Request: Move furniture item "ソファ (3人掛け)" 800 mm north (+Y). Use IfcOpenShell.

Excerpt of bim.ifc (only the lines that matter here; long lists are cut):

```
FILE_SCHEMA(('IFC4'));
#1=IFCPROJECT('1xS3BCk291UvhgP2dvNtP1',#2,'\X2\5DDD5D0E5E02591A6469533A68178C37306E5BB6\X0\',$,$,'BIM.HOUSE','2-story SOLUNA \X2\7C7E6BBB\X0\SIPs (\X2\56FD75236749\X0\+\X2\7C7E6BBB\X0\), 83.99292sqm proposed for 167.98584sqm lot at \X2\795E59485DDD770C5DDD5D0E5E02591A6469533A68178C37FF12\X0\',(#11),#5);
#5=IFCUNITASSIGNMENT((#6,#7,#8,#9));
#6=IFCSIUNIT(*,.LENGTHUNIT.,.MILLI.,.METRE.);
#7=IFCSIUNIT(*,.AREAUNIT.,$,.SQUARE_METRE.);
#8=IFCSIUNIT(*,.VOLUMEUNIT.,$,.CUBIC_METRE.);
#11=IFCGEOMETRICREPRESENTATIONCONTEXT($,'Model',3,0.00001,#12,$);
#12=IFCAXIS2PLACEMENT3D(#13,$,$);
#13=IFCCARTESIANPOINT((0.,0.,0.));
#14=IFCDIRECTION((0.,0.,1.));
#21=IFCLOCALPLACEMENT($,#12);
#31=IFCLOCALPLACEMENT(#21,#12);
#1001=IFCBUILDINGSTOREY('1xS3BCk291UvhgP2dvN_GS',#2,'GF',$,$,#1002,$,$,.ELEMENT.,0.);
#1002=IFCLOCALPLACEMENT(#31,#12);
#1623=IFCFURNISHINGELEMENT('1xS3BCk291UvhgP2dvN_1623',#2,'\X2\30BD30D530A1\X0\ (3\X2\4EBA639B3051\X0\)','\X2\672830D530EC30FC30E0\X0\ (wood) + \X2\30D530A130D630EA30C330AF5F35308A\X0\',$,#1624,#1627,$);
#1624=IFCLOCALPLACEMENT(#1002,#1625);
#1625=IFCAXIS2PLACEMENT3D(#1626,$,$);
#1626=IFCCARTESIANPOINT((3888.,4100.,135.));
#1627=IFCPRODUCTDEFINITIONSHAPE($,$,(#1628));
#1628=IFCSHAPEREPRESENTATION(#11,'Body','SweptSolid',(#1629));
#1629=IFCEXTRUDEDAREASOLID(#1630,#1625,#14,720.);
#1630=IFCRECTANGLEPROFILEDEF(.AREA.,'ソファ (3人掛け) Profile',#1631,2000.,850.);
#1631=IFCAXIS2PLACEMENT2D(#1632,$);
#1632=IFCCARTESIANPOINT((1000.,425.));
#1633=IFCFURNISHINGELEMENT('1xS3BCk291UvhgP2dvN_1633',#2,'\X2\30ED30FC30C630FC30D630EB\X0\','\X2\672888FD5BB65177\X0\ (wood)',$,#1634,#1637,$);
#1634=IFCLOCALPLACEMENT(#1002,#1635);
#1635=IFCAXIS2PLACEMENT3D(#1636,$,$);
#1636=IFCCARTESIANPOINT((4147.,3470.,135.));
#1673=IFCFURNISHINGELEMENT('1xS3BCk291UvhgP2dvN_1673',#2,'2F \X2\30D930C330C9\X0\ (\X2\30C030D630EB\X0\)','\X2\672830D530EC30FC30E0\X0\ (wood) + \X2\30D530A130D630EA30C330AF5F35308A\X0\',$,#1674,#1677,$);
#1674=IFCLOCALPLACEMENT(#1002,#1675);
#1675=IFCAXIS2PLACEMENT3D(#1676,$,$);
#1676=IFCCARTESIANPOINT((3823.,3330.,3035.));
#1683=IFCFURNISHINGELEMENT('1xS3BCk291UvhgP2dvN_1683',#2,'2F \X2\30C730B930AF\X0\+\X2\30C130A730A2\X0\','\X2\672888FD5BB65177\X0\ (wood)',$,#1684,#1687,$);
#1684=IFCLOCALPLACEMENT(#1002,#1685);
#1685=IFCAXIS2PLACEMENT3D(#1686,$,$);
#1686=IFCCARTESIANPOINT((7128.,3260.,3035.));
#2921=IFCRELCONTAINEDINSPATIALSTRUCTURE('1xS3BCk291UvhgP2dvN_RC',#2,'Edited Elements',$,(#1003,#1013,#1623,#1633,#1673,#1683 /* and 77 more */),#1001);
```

```python
import ifcopenshell
import ifcopenshell.api.geometry
import ifcopenshell.util.placement
import ifcopenshell.util.unit

model = ifcopenshell.open("bim.ifc")
unit_scale = ifcopenshell.util.unit.calculate_unit_scale(model)

item = model.by_guid("1xS3BCk291UvhgP2dvN_1623")
matrix = ifcopenshell.util.placement.get_local_placement(item.ObjectPlacement)
matrix[1, 3] += 0.8 / unit_scale
ifcopenshell.api.geometry.edit_object_placement(model, product=item, matrix=matrix, is_si=False)

print(ifcopenshell.util.placement.get_local_placement(item.ObjectPlacement).round(3) + 0.0)

model.write("bim_edited.ifc")
```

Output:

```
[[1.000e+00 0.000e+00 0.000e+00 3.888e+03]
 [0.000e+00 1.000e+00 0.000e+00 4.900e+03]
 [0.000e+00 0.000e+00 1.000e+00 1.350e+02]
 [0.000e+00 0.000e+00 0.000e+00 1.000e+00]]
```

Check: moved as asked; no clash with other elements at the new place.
